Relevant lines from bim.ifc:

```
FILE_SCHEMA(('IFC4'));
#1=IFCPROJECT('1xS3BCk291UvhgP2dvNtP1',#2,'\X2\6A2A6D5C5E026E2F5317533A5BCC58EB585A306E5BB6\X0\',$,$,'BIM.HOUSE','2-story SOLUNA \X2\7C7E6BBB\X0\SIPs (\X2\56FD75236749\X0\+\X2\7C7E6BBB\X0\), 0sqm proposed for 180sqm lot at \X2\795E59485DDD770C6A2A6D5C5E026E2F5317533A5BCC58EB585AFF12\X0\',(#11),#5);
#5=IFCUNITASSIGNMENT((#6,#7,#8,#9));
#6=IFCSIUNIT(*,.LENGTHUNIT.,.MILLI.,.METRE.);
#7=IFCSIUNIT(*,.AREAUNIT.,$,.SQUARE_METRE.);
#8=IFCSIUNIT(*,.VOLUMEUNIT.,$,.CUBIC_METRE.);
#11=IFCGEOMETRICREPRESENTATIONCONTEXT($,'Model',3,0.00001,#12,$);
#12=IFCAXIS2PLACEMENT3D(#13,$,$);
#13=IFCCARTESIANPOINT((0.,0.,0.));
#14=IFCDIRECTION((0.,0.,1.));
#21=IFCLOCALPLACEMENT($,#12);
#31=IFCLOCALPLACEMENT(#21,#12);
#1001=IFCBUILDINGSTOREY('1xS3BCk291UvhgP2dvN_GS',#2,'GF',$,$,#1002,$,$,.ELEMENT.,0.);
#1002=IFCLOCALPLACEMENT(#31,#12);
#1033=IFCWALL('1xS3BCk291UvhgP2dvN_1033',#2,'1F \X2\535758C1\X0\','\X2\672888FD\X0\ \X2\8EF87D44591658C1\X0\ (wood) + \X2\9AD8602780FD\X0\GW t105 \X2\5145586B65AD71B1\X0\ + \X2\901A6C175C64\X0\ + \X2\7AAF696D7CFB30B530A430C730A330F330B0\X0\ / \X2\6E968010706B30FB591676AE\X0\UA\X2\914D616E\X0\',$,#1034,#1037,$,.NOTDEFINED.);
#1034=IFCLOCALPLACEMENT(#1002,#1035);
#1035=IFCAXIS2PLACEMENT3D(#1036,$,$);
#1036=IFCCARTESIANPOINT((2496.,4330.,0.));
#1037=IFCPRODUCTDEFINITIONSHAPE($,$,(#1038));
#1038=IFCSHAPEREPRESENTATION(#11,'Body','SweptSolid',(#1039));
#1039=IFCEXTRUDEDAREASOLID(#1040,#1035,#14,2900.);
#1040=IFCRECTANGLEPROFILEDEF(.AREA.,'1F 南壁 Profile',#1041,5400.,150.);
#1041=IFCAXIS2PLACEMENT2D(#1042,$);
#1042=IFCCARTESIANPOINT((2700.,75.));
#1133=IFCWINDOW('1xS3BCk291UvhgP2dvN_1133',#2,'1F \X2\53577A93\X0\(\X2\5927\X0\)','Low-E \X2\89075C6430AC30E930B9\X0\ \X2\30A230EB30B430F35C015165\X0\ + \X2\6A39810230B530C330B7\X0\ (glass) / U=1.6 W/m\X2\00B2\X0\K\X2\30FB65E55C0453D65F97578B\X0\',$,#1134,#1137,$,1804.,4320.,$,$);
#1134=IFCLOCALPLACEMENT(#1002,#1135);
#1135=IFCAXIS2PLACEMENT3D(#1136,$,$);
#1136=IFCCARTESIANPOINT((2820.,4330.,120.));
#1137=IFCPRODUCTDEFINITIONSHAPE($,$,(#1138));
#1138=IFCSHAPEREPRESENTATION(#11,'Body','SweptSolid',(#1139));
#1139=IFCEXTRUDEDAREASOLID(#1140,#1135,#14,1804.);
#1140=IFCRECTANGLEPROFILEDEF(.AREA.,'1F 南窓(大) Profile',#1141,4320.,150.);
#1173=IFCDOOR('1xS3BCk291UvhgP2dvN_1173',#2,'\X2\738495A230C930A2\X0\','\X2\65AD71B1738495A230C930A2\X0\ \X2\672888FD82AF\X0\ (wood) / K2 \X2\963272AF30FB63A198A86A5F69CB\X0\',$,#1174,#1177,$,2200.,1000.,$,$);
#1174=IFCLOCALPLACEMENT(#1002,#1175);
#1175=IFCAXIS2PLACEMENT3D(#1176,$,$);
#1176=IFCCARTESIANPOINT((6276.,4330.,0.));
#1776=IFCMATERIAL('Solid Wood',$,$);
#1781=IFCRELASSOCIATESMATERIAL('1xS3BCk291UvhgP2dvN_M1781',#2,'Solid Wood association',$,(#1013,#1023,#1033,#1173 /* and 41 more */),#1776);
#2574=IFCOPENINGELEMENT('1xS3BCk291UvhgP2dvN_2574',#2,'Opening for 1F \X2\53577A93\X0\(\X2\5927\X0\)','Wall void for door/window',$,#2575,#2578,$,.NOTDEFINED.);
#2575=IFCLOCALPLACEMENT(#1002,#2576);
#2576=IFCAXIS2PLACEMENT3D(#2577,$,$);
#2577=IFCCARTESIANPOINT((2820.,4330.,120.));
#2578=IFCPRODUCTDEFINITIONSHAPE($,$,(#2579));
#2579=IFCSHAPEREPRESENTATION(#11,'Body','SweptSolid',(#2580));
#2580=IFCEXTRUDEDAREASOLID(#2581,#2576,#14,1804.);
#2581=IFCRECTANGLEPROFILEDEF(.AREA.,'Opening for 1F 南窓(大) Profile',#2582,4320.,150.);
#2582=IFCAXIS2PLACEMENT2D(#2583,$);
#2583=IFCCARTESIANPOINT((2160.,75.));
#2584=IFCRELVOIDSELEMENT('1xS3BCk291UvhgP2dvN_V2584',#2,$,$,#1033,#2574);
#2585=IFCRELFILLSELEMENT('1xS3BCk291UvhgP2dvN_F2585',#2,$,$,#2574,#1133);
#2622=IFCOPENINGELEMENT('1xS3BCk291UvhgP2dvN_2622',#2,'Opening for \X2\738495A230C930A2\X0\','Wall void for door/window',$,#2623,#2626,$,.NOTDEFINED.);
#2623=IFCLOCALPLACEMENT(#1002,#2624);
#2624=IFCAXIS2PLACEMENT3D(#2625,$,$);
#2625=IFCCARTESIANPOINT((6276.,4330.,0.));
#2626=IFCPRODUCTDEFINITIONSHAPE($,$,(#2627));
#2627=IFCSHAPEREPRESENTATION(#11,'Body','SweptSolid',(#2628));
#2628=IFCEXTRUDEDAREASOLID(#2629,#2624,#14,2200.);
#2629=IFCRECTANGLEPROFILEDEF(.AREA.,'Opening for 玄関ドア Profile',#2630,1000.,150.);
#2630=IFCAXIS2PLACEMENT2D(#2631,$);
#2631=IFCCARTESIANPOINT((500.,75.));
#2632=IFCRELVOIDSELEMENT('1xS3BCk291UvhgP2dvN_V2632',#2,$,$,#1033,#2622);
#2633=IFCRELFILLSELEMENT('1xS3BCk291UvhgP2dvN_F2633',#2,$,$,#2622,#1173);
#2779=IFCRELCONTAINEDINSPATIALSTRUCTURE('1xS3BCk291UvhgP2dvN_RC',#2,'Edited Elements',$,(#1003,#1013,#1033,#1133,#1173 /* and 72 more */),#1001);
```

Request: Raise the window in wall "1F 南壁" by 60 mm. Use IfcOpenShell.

```python
import numpy as np
import ifcopenshell
import ifcopenshell.api.geometry
import ifcopenshell.util.placement
import ifcopenshell.util.unit

model = ifcopenshell.open("bim.ifc")
unit_scale = ifcopenshell.util.unit.calculate_unit_scale(model)

window = model.by_id(1133)
opening = window.FillsVoids[0].RelatingOpeningElement
dz = 0.06 / unit_scale

shift = np.array([0.0, 0.0, dz])
# The window is not placed relative to its opening, so move both.
for product in (opening, window):
    matrix = ifcopenshell.util.placement.get_local_placement(product.ObjectPlacement)
    matrix[:3, 3] += shift
    ifcopenshell.api.geometry.edit_object_placement(model, product=product, matrix=matrix, is_si=False)

print(f"moved by {dz * unit_scale:+.3f} m")

model.write("bim_edited.ifc")
```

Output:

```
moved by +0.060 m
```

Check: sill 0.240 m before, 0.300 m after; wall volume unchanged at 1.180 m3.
